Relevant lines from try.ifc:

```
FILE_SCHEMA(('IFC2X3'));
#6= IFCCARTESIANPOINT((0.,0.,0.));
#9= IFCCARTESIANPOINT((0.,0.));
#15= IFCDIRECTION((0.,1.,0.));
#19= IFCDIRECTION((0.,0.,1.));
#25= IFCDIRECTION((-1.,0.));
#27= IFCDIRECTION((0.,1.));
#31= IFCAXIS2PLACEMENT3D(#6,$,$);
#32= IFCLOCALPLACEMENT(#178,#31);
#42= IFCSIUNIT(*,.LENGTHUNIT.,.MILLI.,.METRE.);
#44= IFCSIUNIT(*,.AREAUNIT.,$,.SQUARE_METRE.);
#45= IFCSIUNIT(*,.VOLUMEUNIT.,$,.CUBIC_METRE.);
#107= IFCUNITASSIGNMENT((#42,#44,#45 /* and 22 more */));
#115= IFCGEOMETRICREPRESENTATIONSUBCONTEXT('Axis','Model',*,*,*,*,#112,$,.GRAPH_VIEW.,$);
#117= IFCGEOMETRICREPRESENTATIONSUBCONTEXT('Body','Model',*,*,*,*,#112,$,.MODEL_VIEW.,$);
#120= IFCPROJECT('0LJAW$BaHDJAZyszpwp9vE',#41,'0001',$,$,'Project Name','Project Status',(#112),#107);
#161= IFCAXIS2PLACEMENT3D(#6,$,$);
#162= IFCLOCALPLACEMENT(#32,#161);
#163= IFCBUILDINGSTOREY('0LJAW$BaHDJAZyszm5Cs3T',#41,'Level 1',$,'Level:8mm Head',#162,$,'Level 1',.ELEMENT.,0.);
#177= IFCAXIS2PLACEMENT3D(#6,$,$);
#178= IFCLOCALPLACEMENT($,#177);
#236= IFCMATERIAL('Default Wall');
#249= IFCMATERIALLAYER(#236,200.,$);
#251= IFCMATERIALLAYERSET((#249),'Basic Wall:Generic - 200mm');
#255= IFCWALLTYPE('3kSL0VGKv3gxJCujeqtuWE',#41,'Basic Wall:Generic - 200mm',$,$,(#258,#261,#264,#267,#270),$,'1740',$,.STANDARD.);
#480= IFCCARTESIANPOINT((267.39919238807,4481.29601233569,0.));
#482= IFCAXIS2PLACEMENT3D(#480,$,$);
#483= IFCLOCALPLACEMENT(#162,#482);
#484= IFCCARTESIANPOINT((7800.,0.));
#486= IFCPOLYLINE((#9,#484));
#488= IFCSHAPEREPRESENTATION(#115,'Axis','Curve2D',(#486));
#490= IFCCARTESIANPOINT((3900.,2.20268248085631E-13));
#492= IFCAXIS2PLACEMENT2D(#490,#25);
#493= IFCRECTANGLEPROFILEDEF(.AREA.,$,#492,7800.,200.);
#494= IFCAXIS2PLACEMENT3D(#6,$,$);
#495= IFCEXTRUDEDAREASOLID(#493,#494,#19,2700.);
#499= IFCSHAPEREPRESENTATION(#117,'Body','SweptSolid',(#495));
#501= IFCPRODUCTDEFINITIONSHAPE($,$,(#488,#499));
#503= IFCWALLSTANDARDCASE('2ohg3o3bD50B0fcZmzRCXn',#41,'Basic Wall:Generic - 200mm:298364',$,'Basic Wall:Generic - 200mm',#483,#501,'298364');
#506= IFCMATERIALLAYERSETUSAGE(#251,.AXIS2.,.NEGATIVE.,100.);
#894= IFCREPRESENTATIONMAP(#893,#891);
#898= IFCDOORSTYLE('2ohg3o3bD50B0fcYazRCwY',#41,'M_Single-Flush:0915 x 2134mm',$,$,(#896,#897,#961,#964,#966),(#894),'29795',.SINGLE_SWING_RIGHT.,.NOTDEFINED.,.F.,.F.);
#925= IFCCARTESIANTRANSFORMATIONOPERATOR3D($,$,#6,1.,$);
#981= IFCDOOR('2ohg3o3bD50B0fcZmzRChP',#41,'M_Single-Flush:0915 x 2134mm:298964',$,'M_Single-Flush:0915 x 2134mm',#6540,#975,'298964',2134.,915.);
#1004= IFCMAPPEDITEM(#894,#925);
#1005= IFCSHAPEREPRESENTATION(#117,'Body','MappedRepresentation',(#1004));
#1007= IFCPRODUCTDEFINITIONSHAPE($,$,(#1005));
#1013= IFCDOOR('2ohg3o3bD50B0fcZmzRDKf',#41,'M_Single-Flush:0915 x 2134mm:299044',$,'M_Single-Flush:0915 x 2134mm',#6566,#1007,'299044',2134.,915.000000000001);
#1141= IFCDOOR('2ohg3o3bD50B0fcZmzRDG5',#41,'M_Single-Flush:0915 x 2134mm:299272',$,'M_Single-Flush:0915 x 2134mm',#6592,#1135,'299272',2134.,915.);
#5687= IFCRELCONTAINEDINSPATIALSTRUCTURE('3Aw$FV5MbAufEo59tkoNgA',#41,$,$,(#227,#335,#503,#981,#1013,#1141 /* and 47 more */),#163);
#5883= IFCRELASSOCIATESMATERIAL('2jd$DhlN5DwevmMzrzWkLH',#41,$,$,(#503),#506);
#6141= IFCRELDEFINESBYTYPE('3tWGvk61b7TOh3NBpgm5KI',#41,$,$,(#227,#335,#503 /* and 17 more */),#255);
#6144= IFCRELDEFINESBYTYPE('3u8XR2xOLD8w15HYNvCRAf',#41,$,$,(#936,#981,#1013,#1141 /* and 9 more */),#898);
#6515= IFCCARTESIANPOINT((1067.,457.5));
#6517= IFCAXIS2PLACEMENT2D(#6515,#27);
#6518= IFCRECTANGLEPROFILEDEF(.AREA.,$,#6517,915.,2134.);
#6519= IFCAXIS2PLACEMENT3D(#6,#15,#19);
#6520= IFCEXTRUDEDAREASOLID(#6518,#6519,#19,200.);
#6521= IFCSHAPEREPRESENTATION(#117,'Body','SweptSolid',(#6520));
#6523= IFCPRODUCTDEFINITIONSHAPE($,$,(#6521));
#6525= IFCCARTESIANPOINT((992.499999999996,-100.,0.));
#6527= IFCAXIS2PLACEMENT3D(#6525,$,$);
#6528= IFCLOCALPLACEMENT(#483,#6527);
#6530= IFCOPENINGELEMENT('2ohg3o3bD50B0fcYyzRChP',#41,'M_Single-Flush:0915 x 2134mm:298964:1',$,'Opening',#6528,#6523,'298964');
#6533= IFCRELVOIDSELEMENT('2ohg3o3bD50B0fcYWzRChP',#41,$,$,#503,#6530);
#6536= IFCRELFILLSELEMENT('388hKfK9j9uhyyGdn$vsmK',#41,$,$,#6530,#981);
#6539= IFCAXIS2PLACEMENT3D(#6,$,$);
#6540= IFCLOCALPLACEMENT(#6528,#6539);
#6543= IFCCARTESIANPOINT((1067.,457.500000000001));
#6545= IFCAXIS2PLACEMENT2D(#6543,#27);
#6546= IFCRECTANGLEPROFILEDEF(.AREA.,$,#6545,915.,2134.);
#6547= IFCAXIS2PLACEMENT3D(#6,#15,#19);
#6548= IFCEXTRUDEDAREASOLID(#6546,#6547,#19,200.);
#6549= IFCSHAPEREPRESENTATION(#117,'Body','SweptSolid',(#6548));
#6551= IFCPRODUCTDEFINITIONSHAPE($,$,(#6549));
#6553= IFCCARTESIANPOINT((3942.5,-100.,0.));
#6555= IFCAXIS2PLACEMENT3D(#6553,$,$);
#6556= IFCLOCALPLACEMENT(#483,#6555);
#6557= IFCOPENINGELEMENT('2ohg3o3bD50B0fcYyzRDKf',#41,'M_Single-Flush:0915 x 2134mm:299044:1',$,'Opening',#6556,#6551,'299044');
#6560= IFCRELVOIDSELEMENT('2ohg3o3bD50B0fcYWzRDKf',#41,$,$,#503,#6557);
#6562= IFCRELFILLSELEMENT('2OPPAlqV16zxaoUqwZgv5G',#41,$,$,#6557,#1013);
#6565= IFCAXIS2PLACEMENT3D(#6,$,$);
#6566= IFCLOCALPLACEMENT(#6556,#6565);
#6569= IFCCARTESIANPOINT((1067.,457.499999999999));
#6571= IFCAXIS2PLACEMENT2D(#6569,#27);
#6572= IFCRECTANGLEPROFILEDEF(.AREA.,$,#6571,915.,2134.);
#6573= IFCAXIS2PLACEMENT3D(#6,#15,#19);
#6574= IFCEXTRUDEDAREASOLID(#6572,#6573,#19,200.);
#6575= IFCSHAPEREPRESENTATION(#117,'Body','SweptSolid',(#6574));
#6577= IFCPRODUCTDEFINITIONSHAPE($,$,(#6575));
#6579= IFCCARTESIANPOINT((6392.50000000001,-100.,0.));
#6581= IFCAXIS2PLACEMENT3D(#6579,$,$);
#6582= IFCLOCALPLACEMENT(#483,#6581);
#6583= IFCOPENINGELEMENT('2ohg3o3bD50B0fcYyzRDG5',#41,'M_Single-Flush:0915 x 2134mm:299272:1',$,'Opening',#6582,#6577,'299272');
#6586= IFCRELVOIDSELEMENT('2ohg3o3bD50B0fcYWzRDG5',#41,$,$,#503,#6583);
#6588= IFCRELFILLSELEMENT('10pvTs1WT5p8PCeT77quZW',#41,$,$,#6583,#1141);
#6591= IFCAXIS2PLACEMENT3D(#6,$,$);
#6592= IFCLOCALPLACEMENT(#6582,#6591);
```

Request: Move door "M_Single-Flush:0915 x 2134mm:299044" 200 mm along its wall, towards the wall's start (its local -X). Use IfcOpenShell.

```python
import ifcopenshell
import ifcopenshell.api.geometry
import ifcopenshell.util.placement
import ifcopenshell.util.unit

model = ifcopenshell.open("try.ifc")
unit_scale = ifcopenshell.util.unit.calculate_unit_scale(model)

door = model.by_guid("2ohg3o3bD50B0fcZmzRDKf")
opening = door.FillsVoids[0].RelatingOpeningElement
wall = opening.VoidsElements[0].RelatingBuildingElement

wall_matrix = ifcopenshell.util.placement.get_local_placement(wall.ObjectPlacement)
shift = wall_matrix[:3, 0] * -0.2 / unit_scale
before = ifcopenshell.util.placement.get_local_placement(door.ObjectPlacement)[:3, 3].copy()

# The door is placed relative to its opening, so it follows when the opening moves.
matrix = ifcopenshell.util.placement.get_local_placement(opening.ObjectPlacement)
matrix[:3, 3] += shift
ifcopenshell.api.geometry.edit_object_placement(
    model, product=opening, matrix=matrix, is_si=False, should_transform_children=True
)

after = ifcopenshell.util.placement.get_local_placement(door.ObjectPlacement)[:3, 3]
print("door moved by", (after - before).round(3) + 0.0)

model.write("try_v2.ifc")
```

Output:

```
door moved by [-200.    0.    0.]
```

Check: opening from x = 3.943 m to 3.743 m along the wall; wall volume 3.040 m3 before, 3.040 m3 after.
